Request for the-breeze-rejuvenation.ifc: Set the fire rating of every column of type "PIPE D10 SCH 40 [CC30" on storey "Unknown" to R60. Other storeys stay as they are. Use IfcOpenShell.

First a look at what the model holds.

```python
import ifcopenshell
import ifcopenshell.util.element

model = ifcopenshell.open("the-breeze-rejuvenation.ifc")
print(model.schema)
storey = next(s for s in model.by_type("IfcBuildingStorey") if s.Name == "Unknown")
columns = [e for e in ifcopenshell.util.element.get_decomposition(storey) if e.is_a("IfcColumn")]
seen = {}
for e in columns:
    element_type = ifcopenshell.util.element.get_type(e)
    key = (element_type.Name if element_type != e and element_type else None, ifcopenshell.util.element.get_pset(e, "Pset_ColumnCommon", "FireRating"))
    seen[key] = seen.get(key, 0) + 1
for (name, value), count in sorted(seen.items(), key=str):
    print(count, "x", name, "|", value)
```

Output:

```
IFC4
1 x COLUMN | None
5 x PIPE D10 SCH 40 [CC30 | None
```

```python
import ifcopenshell
import ifcopenshell.api.pset
import ifcopenshell.util.element

model = ifcopenshell.open("the-breeze-rejuvenation.ifc")

storey = next(s for s in model.by_type("IfcBuildingStorey") if s.Name == "Unknown")
columns = [e for e in ifcopenshell.util.element.get_decomposition(storey) if e.is_a("IfcColumn")]

count = 0
for e in columns:
    element_type = ifcopenshell.util.element.get_type(e)
    if element_type in (None, e) or element_type.Name != "PIPE D10 SCH 40 [CC30":
        continue
    found = ifcopenshell.util.element.get_pset(e, "Pset_ColumnCommon", should_inherit=False)
    if found:
        pset = model.by_id(found["id"])
        if len(ifcopenshell.util.element.get_elements_by_pset(pset)) > 1:
            pset = ifcopenshell.api.pset.unshare_pset(model, products=[e], pset=pset)[0]
    else:
        pset = ifcopenshell.api.pset.add_pset(model, product=e, name="Pset_ColumnCommon")
    ifcopenshell.api.pset.edit_pset(model, pset=pset, properties={"FireRating": "R60"})
    count += 1

print(count, "columns updated")

model.write("the-breeze-rejuvenation_edited.ifc")
```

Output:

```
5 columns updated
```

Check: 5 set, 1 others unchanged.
